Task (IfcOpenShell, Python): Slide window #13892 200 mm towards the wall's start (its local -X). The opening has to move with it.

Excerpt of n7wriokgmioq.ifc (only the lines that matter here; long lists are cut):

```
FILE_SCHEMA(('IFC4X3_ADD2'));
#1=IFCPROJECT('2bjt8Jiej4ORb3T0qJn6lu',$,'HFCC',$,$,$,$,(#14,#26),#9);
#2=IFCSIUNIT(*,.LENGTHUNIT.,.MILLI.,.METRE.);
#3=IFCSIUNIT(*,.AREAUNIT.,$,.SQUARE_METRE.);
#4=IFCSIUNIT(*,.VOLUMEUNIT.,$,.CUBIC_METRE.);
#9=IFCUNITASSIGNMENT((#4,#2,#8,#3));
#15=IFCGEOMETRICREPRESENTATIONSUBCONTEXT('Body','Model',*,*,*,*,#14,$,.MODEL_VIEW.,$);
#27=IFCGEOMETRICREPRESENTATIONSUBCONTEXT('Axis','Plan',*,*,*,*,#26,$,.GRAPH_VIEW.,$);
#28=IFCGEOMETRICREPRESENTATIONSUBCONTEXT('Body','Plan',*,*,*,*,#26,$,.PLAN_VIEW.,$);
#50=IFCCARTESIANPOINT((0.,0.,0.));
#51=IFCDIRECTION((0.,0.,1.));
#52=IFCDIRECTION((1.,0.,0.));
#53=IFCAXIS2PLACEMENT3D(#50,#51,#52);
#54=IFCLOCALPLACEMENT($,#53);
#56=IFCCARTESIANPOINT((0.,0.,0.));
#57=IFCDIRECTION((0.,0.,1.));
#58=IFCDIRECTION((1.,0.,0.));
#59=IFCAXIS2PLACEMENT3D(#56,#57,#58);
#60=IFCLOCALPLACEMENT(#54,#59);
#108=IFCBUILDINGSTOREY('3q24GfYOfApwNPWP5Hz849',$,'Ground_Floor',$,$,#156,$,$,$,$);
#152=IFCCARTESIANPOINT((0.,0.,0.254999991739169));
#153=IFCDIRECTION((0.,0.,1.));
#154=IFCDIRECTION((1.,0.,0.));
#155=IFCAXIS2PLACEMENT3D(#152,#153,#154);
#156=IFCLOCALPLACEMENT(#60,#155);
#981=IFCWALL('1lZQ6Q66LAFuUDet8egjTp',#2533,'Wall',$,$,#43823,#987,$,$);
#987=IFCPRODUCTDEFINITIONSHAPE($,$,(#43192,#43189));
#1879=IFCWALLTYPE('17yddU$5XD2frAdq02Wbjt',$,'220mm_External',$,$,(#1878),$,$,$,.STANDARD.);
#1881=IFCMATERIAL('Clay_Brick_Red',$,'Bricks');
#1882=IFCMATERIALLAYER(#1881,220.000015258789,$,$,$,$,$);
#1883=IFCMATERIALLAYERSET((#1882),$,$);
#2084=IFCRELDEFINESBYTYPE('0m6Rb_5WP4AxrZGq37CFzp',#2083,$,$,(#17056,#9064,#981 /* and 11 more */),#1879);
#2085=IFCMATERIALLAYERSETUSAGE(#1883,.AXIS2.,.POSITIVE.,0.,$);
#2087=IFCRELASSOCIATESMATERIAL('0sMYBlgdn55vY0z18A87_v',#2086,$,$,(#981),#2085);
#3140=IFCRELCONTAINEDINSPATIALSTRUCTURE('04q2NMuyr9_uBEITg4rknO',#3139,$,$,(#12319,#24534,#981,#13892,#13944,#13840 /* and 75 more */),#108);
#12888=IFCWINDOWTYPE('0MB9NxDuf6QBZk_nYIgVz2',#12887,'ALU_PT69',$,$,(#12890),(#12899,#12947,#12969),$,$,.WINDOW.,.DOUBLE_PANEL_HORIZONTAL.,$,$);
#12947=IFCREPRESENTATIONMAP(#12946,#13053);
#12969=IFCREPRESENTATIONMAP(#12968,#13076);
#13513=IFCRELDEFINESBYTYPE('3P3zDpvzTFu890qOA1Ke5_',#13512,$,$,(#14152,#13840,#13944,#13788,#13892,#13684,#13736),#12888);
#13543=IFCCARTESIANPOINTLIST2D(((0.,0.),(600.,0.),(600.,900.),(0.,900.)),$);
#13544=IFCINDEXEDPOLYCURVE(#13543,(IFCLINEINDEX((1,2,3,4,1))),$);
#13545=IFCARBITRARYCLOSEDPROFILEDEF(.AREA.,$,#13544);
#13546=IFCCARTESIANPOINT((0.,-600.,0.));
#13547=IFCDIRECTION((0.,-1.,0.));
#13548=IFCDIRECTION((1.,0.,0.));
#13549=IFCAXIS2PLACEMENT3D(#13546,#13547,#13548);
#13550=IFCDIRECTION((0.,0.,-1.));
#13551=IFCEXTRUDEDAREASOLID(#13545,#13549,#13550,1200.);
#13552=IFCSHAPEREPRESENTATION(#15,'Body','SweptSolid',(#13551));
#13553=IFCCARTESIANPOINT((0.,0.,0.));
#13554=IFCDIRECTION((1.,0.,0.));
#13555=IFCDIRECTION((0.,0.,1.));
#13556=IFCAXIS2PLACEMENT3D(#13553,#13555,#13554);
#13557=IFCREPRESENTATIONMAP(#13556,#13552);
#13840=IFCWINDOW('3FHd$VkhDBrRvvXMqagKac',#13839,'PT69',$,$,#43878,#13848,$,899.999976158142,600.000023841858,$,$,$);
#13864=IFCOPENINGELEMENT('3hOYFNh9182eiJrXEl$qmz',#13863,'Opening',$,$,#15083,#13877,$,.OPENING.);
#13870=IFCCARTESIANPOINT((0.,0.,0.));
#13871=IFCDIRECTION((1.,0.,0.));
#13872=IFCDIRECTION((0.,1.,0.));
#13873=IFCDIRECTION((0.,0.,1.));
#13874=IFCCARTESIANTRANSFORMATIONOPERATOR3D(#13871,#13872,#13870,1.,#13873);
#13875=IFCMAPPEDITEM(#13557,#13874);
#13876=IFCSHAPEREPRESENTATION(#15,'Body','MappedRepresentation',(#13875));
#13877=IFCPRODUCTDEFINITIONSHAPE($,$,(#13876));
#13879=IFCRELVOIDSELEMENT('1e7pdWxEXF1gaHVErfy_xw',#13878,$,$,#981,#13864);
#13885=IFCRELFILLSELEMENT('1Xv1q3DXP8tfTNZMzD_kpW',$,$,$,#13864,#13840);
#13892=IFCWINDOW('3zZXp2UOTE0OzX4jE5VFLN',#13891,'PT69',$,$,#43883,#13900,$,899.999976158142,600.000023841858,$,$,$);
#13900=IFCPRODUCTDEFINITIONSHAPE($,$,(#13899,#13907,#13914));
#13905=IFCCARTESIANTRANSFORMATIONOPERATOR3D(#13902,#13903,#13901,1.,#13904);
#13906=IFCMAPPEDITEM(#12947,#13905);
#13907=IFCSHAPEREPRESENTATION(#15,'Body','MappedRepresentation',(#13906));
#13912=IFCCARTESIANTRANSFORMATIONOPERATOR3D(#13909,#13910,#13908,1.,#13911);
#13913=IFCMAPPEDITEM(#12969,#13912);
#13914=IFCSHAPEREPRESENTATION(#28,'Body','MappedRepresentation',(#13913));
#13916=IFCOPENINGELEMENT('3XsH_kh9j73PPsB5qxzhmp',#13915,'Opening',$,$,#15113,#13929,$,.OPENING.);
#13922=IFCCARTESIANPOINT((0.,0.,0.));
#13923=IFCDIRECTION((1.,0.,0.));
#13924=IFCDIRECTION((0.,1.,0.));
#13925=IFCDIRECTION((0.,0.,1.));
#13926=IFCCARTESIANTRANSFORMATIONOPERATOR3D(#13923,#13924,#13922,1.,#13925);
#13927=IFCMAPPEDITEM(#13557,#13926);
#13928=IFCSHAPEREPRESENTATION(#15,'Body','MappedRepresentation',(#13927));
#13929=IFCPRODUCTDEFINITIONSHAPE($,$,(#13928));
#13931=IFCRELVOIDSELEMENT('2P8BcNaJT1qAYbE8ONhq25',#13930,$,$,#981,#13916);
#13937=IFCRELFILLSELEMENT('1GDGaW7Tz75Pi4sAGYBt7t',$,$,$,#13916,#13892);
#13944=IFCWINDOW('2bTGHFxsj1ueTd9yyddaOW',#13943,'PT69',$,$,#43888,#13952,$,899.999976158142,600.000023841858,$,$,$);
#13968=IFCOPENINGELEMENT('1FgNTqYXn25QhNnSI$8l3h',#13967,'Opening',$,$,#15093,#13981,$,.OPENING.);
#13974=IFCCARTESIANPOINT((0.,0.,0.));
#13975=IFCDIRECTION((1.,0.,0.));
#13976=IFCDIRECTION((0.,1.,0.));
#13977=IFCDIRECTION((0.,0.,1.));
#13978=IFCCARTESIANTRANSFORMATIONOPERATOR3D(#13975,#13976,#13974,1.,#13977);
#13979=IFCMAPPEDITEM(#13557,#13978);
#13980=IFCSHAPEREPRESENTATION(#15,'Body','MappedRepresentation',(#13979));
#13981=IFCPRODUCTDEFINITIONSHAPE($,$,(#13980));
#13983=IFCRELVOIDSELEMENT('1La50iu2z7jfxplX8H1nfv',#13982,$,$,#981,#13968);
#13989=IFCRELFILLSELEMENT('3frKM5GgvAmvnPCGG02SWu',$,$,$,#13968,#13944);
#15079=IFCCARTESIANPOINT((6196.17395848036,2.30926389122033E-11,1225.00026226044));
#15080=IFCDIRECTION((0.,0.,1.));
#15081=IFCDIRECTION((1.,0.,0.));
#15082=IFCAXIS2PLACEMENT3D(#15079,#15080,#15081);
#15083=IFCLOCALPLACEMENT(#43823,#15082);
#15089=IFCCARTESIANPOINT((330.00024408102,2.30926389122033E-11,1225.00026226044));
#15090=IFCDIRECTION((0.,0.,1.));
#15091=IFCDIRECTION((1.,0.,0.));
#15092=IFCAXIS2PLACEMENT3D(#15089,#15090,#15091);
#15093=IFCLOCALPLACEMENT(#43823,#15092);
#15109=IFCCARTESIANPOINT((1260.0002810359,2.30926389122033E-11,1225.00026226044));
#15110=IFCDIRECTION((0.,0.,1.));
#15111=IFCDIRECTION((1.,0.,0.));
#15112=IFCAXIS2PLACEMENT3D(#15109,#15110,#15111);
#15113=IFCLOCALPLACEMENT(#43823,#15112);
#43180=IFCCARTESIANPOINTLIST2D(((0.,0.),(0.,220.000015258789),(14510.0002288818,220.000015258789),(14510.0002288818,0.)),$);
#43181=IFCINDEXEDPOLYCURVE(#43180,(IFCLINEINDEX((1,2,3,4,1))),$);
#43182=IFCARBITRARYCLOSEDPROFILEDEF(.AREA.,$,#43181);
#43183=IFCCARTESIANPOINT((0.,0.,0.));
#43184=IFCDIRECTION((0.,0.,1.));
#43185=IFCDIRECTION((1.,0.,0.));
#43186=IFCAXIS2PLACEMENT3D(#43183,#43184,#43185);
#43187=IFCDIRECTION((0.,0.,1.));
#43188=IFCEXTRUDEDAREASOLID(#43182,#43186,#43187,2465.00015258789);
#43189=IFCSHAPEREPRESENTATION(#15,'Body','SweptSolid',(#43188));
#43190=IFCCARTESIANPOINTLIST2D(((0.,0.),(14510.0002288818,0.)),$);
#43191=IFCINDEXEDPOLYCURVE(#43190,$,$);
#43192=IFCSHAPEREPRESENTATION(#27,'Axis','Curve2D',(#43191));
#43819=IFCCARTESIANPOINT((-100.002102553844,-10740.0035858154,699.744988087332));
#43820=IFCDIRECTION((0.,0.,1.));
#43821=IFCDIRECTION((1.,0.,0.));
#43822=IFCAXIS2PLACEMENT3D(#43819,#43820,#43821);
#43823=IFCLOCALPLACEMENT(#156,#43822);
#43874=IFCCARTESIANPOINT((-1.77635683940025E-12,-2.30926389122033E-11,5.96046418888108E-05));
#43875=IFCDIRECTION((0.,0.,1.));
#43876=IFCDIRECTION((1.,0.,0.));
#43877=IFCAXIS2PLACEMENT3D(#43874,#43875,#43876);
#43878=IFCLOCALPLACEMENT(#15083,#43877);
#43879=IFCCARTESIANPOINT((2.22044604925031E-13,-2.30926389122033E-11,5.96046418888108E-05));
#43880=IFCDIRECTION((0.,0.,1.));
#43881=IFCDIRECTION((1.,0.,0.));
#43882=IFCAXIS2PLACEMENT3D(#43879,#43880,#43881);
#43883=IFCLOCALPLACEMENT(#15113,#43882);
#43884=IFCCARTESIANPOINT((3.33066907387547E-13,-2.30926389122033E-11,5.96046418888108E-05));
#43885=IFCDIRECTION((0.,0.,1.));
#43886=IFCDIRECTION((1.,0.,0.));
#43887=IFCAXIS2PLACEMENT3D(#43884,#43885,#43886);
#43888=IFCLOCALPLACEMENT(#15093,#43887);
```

```python
import ifcopenshell
import ifcopenshell.api.geometry
import ifcopenshell.util.placement

model = ifcopenshell.open("n7wriokgmioq.ifc")

window = model.by_id(13892)
opening = window.FillsVoids[0].RelatingOpeningElement
wall = opening.VoidsElements[0].RelatingBuildingElement

wall_matrix = ifcopenshell.util.placement.get_local_placement(wall.ObjectPlacement)
shift = wall_matrix[:3, 0] * -200.0
before = ifcopenshell.util.placement.get_local_placement(window.ObjectPlacement)[:3, 3].copy()

# The window is placed relative to its opening, so it follows when the opening moves.
matrix = ifcopenshell.util.placement.get_local_placement(opening.ObjectPlacement)
matrix[:3, 3] += shift
ifcopenshell.api.geometry.edit_object_placement(
    model, product=opening, matrix=matrix, is_si=False, should_transform_children=True
)

after = ifcopenshell.util.placement.get_local_placement(window.ObjectPlacement)[:3, 3]
print("window moved by", (after - before).round(3) + 0.0)

model.write("n7wriokgmioq-out.ifc")
```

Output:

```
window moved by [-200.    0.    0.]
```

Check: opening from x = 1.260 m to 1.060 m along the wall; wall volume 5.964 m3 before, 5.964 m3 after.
